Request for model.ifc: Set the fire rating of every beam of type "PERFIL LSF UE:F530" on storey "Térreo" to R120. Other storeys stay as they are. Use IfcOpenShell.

First a look at what the model holds.

```python
import ifcopenshell
import ifcopenshell.util.element

model = ifcopenshell.open("model.ifc")
print(model.schema)
storey = next(s for s in model.by_type("IfcBuildingStorey") if s.Name == "Térreo")
beams = [e for e in ifcopenshell.util.element.get_decomposition(storey) if e.is_a("IfcBeam")]
seen = {}
for e in beams:
    element_type = ifcopenshell.util.element.get_type(e)
    key = (element_type.Name if element_type != e and element_type else None, ifcopenshell.util.element.get_pset(e, "Pset_BeamCommon", "FireRating"))
    seen[key] = seen.get(key, 0) + 1
for (name, value), count in sorted(seen.items(), key=str):
    print(count, "x", name, "|", value)
```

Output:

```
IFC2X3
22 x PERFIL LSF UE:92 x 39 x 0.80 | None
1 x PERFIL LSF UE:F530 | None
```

```python
import ifcopenshell
import ifcopenshell.api.pset
import ifcopenshell.util.element

model = ifcopenshell.open("model.ifc")

storey = next(s for s in model.by_type("IfcBuildingStorey") if s.Name == "Térreo")
beams = [e for e in ifcopenshell.util.element.get_decomposition(storey) if e.is_a("IfcBeam")]

count = 0
for e in beams:
    element_type = ifcopenshell.util.element.get_type(e)
    if element_type in (None, e) or element_type.Name != "PERFIL LSF UE:F530":
        continue
    # add_pset returns the element's existing set when there is one.
    pset = ifcopenshell.api.pset.add_pset(model, product=e, name="Pset_BeamCommon")
    ifcopenshell.api.pset.edit_pset(model, pset=pset, properties={"FireRating": "R120"})
    count += 1

print(count, "beams updated")

model.write("model_edited.ifc")
```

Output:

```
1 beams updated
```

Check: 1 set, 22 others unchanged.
